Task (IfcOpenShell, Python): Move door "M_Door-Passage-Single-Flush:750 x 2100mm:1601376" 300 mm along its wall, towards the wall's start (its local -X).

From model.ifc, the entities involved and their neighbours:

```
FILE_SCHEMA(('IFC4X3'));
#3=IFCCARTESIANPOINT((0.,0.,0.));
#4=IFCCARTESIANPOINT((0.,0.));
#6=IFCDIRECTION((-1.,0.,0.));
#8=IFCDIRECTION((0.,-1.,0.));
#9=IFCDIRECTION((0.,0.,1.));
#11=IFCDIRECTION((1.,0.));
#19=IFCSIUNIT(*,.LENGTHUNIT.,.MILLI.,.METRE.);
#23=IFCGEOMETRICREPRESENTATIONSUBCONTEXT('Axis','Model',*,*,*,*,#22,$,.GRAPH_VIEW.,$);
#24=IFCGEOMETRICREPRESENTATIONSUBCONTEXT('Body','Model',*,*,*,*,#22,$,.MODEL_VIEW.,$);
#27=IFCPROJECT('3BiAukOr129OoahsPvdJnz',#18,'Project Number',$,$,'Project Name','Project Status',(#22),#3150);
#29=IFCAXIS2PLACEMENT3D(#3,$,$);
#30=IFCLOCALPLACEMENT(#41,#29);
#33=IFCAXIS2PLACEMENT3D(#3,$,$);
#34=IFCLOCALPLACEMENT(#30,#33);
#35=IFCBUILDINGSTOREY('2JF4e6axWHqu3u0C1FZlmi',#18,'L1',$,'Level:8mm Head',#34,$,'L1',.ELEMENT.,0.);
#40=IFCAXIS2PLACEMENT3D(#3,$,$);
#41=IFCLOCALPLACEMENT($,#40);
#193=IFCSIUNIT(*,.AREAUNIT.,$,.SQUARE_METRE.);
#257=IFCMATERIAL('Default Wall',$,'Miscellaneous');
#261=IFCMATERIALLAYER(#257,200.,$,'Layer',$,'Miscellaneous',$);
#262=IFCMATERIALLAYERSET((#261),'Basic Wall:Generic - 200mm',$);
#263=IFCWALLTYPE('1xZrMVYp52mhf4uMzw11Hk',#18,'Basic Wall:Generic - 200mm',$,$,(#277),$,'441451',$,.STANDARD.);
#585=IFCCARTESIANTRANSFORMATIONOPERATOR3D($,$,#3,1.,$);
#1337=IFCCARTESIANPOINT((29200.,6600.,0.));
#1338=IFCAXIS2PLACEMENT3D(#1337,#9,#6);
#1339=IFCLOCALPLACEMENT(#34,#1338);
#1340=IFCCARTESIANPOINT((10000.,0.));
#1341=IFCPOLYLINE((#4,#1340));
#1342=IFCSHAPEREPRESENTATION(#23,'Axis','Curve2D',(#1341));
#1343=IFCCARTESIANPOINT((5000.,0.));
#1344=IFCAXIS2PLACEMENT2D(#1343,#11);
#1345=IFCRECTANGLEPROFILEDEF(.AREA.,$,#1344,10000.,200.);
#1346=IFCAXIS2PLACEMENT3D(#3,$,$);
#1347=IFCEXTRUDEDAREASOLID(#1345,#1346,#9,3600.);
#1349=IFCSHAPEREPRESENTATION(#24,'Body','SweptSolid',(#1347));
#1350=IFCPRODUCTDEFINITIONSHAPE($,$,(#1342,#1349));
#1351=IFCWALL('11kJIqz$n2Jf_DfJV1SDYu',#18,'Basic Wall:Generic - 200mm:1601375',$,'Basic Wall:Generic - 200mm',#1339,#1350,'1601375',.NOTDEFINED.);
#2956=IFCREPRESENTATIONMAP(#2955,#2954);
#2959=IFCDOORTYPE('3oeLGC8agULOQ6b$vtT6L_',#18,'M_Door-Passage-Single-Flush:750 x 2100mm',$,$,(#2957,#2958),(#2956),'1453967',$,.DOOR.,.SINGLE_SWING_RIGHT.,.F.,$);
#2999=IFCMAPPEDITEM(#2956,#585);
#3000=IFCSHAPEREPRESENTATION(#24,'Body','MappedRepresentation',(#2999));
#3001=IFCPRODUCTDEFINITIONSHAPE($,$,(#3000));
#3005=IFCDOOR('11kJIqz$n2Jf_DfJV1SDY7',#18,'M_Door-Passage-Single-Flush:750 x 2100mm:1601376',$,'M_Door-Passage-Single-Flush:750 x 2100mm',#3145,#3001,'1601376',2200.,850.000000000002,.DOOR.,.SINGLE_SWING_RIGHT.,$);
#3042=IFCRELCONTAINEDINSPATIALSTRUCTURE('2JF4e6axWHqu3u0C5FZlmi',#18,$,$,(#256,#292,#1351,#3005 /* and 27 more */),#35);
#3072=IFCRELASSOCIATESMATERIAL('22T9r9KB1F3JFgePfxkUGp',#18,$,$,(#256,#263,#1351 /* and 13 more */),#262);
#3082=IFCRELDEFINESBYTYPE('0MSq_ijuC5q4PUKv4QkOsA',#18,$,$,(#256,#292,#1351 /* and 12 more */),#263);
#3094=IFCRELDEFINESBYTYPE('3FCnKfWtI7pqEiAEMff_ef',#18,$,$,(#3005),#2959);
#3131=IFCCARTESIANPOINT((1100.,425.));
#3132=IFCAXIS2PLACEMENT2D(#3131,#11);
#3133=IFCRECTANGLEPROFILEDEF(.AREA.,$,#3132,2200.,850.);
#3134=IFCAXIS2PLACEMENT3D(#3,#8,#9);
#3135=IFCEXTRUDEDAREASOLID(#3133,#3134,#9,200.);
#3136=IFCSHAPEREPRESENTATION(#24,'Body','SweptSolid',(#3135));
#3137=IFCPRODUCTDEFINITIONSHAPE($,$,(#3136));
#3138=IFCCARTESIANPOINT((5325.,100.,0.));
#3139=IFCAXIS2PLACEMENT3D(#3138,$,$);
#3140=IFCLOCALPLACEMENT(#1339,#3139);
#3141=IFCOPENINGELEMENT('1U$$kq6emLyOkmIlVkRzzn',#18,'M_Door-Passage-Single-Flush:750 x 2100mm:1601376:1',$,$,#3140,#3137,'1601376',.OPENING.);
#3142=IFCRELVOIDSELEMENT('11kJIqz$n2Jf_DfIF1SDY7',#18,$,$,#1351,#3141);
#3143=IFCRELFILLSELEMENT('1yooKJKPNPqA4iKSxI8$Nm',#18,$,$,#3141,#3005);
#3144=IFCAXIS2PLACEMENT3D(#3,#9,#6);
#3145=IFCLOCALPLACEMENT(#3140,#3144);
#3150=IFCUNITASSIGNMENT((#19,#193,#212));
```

```python
import ifcopenshell
import ifcopenshell.api.geometry
import ifcopenshell.util.placement
import ifcopenshell.util.unit

model = ifcopenshell.open("model.ifc")
unit_scale = ifcopenshell.util.unit.calculate_unit_scale(model)

door = model.by_guid("11kJIqz$n2Jf_DfJV1SDY7")
opening = door.FillsVoids[0].RelatingOpeningElement
wall = opening.VoidsElements[0].RelatingBuildingElement

wall_matrix = ifcopenshell.util.placement.get_local_placement(wall.ObjectPlacement)
shift = wall_matrix[:3, 0] * -0.3 / unit_scale
before = ifcopenshell.util.placement.get_local_placement(door.ObjectPlacement)[:3, 3].copy()

# The door is placed relative to its opening, so it follows when the opening moves.
matrix = ifcopenshell.util.placement.get_local_placement(opening.ObjectPlacement)
matrix[:3, 3] += shift
ifcopenshell.api.geometry.edit_object_placement(
    model, product=opening, matrix=matrix, is_si=False, should_transform_children=True
)

after = ifcopenshell.util.placement.get_local_placement(door.ObjectPlacement)[:3, 3]
print("door moved by", (after - before).round(3) + 0.0)

model.write("model_v2.ifc")
```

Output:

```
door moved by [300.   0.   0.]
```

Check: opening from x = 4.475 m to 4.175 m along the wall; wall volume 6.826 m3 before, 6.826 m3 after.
